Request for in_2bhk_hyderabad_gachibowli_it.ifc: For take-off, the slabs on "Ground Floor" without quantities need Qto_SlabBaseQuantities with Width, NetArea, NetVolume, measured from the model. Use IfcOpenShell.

First a look at what the model holds.

```python
import ifcopenshell
import ifcopenshell.util.element
import ifcopenshell.util.unit

model = ifcopenshell.open("in_2bhk_hyderabad_gachibowli_it.ifc")
print(model.schema)
for unit_type in ("LENGTHUNIT", "AREAUNIT", "VOLUMEUNIT"):
    print(unit_type, ifcopenshell.util.unit.calculate_unit_scale(model, unit_type))
storey = next(s for s in model.by_type("IfcBuildingStorey") if s.Name == "Ground Floor")
slabs = [e for e in ifcopenshell.util.element.get_decomposition(storey) if e.is_a("IfcSlab")]
for e in sorted(slabs, key=lambda e: e.id()):
    print(e.id(), e.is_a(), e.Name, list(ifcopenshell.util.element.get_psets(e, qtos_only=True)), sep=" | ")
```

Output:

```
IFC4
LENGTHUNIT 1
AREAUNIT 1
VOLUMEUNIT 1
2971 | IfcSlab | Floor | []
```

```python
import ifcopenshell
import ifcopenshell.api.pset
import ifcopenshell.geom
import ifcopenshell.util.element
import ifcopenshell.util.shape
import ifcopenshell.util.unit

model = ifcopenshell.open("in_2bhk_hyderabad_gachibowli_it.ifc")
unit_scale = ifcopenshell.util.unit.calculate_unit_scale(model)
area_scale = ifcopenshell.util.unit.calculate_unit_scale(model, "AREAUNIT")
volume_scale = ifcopenshell.util.unit.calculate_unit_scale(model, "VOLUMEUNIT")
settings = ifcopenshell.geom.settings()

storey = next(s for s in model.by_type("IfcBuildingStorey") if s.Name == "Ground Floor")
slabs = [e for e in ifcopenshell.util.element.get_decomposition(storey) if e.is_a("IfcSlab")]

for e in sorted(slabs, key=lambda e: e.id()):
    if ifcopenshell.util.element.get_psets(e, qtos_only=True, should_inherit=False):
        continue
    # Geometry comes back in metres, in the element's own axes.
    shape = ifcopenshell.geom.create_shape(settings, e)
    values = {
        "Width": ifcopenshell.util.shape.get_z(shape.geometry) / unit_scale,
        "NetArea": ifcopenshell.util.shape.get_footprint_area(shape.geometry) / area_scale,
        "NetVolume": ifcopenshell.util.shape.get_volume(shape.geometry) / volume_scale,
    }
    qto = ifcopenshell.api.pset.add_qto(model, product=e, name="Qto_SlabBaseQuantities")
    ifcopenshell.api.pset.edit_qto(model, qto=qto, properties=values)
    print(e.id(), {k: round(v, 3) for k, v in values.items()})

model.write("in_2bhk_hyderabad_gachibowli_it_edited.ifc")
```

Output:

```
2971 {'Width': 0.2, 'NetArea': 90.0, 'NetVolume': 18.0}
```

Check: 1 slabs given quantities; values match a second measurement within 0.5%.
